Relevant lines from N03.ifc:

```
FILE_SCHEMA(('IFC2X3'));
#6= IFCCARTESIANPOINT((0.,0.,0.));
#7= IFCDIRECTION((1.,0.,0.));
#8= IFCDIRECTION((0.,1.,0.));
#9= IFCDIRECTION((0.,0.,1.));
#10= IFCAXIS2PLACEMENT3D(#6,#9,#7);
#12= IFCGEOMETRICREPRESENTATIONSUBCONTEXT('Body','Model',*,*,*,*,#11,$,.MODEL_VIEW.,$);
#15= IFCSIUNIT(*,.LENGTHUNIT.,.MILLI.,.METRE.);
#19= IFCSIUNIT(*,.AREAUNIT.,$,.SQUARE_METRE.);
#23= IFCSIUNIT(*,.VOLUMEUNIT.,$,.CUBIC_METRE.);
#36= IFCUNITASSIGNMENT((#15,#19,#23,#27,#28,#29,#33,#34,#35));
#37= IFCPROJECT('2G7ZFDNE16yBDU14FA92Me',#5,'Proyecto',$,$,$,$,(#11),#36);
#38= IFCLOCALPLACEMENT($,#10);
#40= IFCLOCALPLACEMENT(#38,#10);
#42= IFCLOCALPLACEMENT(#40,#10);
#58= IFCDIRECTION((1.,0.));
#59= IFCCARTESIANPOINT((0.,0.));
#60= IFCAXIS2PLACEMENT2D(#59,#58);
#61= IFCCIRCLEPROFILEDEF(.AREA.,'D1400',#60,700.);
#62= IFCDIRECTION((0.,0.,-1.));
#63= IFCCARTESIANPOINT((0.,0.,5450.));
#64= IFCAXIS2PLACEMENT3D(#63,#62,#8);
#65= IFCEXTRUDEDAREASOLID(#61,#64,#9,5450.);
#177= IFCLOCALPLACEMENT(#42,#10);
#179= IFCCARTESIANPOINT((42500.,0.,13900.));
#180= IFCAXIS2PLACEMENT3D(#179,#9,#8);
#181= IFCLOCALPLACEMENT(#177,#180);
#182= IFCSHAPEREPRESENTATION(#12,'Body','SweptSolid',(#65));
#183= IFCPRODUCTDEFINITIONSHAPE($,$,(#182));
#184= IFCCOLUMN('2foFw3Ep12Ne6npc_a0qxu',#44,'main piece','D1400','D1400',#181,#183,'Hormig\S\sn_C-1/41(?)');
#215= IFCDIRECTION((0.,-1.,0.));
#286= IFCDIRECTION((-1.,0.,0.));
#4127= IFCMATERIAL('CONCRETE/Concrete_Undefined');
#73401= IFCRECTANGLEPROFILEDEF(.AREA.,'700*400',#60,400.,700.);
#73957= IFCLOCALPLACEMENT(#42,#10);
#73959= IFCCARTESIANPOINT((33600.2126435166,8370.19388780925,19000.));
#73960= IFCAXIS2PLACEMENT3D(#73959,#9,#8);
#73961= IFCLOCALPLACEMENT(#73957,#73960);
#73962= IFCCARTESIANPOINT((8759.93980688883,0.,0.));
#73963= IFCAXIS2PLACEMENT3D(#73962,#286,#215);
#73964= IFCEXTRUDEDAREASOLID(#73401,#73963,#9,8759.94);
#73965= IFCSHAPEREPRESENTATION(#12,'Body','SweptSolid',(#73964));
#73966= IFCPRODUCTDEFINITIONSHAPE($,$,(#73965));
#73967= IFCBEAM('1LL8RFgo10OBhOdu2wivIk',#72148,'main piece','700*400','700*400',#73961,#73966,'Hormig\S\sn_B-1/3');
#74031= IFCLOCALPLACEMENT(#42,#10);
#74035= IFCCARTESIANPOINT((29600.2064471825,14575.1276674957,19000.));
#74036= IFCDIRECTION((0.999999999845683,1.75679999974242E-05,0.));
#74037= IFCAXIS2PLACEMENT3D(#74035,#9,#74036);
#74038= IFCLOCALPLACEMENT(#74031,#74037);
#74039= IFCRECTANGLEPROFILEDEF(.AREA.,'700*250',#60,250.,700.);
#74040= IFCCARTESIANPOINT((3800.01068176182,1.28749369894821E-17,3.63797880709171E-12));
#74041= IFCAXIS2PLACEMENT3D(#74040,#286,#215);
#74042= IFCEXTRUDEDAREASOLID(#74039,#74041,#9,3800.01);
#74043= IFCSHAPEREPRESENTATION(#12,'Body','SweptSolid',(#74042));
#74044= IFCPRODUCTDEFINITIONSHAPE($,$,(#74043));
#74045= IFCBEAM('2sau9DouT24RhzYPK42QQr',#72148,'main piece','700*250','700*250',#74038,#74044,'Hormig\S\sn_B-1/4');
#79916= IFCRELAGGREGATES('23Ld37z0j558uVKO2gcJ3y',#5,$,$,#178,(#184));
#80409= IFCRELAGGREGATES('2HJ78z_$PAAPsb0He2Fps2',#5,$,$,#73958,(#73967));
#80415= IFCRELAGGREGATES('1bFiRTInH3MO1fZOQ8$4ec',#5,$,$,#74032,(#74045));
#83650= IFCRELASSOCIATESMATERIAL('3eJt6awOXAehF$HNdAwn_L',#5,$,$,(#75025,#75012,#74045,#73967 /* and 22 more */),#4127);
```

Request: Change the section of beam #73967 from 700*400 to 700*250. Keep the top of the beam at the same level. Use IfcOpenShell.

```python
import ifcopenshell
import ifcopenshell.util.element
import ifcopenshell.util.representation

model = ifcopenshell.open("N03.ifc")

member = model.by_guid("1LL8RFgo10OBhOdu2wivIk")
source = next(p for p in model.by_type("IfcRectangleProfileDef") if p.ProfileName == "700*250")

body = ifcopenshell.util.representation.get_representation(member, "Model", "Body")
solid = body.Items[0]
old_profile = solid.SweptArea

# Copy the section's sizes but keep this member's own profile position.
profile = ifcopenshell.util.element.copy(model, source)
# Profiles are centred, so shift by half the change in depth to hold the top.
shift = (old_profile.YDim - profile.YDim) / 2
x, y = old_profile.Position.Location.Coordinates
up = (0.0, 1.0)  # upwards, in the solid's own plane
location = model.createIfcCartesianPoint((x + up[0] * shift, y + up[1] * shift))
profile.Position = model.createIfcAxis2Placement2D(location, old_profile.Position.RefDirection)
solid.SweptArea = profile
if not model.get_total_inverses(old_profile):
    ifcopenshell.util.element.remove_deep2(model, old_profile)
member.Description = member.Description.replace("700*400", "700*250")
member.ObjectType = member.ObjectType.replace("700*400", "700*250")

print(solid.SweptArea)

model.write("N03_rev.ifc")
```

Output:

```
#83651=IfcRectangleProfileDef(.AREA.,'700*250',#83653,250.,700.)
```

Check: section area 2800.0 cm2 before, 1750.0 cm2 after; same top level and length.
